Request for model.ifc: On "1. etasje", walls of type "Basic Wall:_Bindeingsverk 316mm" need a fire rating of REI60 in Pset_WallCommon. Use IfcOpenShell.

First a look at what the model holds.

```python
import ifcopenshell
import ifcopenshell.util.element

model = ifcopenshell.open("model.ifc")
print(model.schema)
storey = next(s for s in model.by_type("IfcBuildingStorey") if s.Name == "1. etasje")
walls = [e for e in ifcopenshell.util.element.get_decomposition(storey) if e.is_a("IfcWall")]
seen = {}
for e in walls:
    element_type = ifcopenshell.util.element.get_type(e)
    key = (element_type.Name if element_type != e and element_type else None, ifcopenshell.util.element.get_pset(e, "Pset_WallCommon", "FireRating"))
    seen[key] = seen.get(key, 0) + 1
for (name, value), count in sorted(seen.items(), key=str):
    print(count, "x", name, "|", value)
```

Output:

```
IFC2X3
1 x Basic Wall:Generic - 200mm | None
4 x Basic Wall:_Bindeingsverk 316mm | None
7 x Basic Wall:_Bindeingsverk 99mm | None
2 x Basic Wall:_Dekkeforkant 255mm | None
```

```python
import ifcopenshell
import ifcopenshell.api.pset
import ifcopenshell.util.element

model = ifcopenshell.open("model.ifc")

storey = next(s for s in model.by_type("IfcBuildingStorey") if s.Name == "1. etasje")
walls = [e for e in ifcopenshell.util.element.get_decomposition(storey) if e.is_a("IfcWall")]

count = 0
for e in walls:
    element_type = ifcopenshell.util.element.get_type(e)
    if element_type in (None, e) or element_type.Name != "Basic Wall:_Bindeingsverk 316mm":
        continue
    # add_pset returns the element's existing set when there is one.
    pset = ifcopenshell.api.pset.add_pset(model, product=e, name="Pset_WallCommon")
    ifcopenshell.api.pset.edit_pset(model, pset=pset, properties={"FireRating": "REI60"})
    count += 1

print(count, "walls updated")

model.write("model_rev.ifc")
```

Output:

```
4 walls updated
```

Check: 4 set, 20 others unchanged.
